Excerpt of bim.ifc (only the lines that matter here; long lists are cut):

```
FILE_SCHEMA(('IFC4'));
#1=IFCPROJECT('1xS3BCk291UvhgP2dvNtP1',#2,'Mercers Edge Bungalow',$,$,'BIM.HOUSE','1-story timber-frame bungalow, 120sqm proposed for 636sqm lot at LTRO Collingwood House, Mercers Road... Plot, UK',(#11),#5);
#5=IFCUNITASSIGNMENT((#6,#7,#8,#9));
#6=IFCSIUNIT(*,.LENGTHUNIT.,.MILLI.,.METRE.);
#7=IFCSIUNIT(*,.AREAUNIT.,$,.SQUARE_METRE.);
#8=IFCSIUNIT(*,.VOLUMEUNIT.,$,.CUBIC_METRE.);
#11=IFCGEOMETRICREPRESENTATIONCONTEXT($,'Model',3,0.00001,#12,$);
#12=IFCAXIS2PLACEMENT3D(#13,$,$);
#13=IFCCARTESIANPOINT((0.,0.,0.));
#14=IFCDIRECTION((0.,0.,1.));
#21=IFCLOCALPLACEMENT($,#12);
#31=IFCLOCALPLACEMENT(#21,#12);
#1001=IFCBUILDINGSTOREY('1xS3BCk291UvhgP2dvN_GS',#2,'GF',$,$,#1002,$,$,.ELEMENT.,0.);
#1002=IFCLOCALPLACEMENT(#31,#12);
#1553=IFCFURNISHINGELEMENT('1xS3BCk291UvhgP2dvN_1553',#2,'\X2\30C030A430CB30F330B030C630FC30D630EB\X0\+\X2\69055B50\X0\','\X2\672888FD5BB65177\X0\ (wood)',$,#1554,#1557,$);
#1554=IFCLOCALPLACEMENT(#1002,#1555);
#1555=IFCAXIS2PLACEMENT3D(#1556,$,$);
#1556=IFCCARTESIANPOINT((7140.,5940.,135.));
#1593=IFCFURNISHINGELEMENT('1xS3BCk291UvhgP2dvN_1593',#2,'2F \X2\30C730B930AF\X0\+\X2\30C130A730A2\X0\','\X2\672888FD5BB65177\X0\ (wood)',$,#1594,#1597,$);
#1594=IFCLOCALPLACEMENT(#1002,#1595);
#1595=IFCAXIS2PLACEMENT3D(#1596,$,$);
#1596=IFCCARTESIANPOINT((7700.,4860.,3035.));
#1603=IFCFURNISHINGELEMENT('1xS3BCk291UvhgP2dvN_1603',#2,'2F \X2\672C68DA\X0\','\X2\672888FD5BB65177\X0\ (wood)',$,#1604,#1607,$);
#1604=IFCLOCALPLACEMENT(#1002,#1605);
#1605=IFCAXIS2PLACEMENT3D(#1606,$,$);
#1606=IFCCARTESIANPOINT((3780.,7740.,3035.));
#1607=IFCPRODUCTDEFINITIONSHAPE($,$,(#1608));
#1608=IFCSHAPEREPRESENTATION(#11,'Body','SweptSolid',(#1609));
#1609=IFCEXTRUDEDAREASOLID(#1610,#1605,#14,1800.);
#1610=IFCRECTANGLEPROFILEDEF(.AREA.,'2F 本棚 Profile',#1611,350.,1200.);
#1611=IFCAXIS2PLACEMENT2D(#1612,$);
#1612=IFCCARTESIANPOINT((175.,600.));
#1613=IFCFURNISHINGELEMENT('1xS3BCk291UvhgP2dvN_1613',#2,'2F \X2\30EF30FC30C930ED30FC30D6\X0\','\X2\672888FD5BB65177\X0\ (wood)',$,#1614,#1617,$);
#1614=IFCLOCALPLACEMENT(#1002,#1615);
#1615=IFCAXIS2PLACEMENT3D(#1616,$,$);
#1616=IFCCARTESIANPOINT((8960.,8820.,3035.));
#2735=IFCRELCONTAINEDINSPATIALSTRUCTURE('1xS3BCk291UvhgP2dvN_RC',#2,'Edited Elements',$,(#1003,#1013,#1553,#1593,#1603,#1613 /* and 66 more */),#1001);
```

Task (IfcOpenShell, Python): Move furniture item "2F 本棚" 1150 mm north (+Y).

```python
import ifcopenshell
import ifcopenshell.api.geometry
import ifcopenshell.util.placement

model = ifcopenshell.open("bim.ifc")

item = model.by_id(1603)
matrix = ifcopenshell.util.placement.get_local_placement(item.ObjectPlacement)
matrix[1, 3] += 1150.0
ifcopenshell.api.geometry.edit_object_placement(model, product=item, matrix=matrix, is_si=False)

print(ifcopenshell.util.placement.get_local_placement(item.ObjectPlacement).round(3) + 0.0)

model.write("bim_rev.ifc")
```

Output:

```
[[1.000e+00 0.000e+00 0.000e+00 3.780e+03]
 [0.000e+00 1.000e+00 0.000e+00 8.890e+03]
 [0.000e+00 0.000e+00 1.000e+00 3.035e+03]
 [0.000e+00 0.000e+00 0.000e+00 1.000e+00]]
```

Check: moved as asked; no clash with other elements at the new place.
